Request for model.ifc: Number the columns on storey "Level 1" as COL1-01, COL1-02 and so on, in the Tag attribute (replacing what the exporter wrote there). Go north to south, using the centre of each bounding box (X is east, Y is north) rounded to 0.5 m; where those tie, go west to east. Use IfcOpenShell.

First a look at what the model holds.

```python
import ifcopenshell
import ifcopenshell.util.element
import ifcopenshell.util.placement

model = ifcopenshell.open("model.ifc")
print(model.schema)
storey = next(s for s in model.by_type("IfcBuildingStorey") if s.Name == "Level 1")
columns = [e for e in ifcopenshell.util.element.get_decomposition(storey) if e.is_a("IfcColumn")]
for e in sorted(columns, key=lambda e: e.id()):
    origin = ifcopenshell.util.placement.get_local_placement(e.ObjectPlacement)[:3, 3]
    print(e.id(), e.Tag, e.Name, origin.round(2) + 0.0, sep=" | ")
```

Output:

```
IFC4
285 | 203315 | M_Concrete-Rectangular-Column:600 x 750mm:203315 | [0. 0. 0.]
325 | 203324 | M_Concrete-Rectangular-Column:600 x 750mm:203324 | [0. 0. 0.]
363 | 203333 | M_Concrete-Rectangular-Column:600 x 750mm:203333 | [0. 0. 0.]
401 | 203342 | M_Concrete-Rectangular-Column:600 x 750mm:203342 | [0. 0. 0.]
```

```python
import ifcopenshell
import ifcopenshell.geom
import ifcopenshell.util.element
import ifcopenshell.util.shape

model = ifcopenshell.open("model.ifc")
settings = ifcopenshell.geom.settings()
settings.set("use-world-coords", True)


def centre(element):
    shape = ifcopenshell.geom.create_shape(settings, element)
    return ifcopenshell.util.shape.get_bbox_centroid(shape.geometry)


storey = next(s for s in model.by_type("IfcBuildingStorey") if s.Name == "Level 1")
columns = [e for e in ifcopenshell.util.element.get_decomposition(storey) if e.is_a("IfcColumn")]

# Insertion points can sit at a corner or the storey origin, so sort by the geometry (in metres).
centres = {e: centre(e) for e in columns}
columns.sort(key=lambda e: (-round(centres[e][1] / 0.5), centres[e][0]))

for i, e in enumerate(columns, start=1):
    number = f"COL1-{i:02d}"
    e.Tag = number
    print(e.id(), number)

model.write("model_rev.ifc")
```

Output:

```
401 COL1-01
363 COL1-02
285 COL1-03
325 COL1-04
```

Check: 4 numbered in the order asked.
